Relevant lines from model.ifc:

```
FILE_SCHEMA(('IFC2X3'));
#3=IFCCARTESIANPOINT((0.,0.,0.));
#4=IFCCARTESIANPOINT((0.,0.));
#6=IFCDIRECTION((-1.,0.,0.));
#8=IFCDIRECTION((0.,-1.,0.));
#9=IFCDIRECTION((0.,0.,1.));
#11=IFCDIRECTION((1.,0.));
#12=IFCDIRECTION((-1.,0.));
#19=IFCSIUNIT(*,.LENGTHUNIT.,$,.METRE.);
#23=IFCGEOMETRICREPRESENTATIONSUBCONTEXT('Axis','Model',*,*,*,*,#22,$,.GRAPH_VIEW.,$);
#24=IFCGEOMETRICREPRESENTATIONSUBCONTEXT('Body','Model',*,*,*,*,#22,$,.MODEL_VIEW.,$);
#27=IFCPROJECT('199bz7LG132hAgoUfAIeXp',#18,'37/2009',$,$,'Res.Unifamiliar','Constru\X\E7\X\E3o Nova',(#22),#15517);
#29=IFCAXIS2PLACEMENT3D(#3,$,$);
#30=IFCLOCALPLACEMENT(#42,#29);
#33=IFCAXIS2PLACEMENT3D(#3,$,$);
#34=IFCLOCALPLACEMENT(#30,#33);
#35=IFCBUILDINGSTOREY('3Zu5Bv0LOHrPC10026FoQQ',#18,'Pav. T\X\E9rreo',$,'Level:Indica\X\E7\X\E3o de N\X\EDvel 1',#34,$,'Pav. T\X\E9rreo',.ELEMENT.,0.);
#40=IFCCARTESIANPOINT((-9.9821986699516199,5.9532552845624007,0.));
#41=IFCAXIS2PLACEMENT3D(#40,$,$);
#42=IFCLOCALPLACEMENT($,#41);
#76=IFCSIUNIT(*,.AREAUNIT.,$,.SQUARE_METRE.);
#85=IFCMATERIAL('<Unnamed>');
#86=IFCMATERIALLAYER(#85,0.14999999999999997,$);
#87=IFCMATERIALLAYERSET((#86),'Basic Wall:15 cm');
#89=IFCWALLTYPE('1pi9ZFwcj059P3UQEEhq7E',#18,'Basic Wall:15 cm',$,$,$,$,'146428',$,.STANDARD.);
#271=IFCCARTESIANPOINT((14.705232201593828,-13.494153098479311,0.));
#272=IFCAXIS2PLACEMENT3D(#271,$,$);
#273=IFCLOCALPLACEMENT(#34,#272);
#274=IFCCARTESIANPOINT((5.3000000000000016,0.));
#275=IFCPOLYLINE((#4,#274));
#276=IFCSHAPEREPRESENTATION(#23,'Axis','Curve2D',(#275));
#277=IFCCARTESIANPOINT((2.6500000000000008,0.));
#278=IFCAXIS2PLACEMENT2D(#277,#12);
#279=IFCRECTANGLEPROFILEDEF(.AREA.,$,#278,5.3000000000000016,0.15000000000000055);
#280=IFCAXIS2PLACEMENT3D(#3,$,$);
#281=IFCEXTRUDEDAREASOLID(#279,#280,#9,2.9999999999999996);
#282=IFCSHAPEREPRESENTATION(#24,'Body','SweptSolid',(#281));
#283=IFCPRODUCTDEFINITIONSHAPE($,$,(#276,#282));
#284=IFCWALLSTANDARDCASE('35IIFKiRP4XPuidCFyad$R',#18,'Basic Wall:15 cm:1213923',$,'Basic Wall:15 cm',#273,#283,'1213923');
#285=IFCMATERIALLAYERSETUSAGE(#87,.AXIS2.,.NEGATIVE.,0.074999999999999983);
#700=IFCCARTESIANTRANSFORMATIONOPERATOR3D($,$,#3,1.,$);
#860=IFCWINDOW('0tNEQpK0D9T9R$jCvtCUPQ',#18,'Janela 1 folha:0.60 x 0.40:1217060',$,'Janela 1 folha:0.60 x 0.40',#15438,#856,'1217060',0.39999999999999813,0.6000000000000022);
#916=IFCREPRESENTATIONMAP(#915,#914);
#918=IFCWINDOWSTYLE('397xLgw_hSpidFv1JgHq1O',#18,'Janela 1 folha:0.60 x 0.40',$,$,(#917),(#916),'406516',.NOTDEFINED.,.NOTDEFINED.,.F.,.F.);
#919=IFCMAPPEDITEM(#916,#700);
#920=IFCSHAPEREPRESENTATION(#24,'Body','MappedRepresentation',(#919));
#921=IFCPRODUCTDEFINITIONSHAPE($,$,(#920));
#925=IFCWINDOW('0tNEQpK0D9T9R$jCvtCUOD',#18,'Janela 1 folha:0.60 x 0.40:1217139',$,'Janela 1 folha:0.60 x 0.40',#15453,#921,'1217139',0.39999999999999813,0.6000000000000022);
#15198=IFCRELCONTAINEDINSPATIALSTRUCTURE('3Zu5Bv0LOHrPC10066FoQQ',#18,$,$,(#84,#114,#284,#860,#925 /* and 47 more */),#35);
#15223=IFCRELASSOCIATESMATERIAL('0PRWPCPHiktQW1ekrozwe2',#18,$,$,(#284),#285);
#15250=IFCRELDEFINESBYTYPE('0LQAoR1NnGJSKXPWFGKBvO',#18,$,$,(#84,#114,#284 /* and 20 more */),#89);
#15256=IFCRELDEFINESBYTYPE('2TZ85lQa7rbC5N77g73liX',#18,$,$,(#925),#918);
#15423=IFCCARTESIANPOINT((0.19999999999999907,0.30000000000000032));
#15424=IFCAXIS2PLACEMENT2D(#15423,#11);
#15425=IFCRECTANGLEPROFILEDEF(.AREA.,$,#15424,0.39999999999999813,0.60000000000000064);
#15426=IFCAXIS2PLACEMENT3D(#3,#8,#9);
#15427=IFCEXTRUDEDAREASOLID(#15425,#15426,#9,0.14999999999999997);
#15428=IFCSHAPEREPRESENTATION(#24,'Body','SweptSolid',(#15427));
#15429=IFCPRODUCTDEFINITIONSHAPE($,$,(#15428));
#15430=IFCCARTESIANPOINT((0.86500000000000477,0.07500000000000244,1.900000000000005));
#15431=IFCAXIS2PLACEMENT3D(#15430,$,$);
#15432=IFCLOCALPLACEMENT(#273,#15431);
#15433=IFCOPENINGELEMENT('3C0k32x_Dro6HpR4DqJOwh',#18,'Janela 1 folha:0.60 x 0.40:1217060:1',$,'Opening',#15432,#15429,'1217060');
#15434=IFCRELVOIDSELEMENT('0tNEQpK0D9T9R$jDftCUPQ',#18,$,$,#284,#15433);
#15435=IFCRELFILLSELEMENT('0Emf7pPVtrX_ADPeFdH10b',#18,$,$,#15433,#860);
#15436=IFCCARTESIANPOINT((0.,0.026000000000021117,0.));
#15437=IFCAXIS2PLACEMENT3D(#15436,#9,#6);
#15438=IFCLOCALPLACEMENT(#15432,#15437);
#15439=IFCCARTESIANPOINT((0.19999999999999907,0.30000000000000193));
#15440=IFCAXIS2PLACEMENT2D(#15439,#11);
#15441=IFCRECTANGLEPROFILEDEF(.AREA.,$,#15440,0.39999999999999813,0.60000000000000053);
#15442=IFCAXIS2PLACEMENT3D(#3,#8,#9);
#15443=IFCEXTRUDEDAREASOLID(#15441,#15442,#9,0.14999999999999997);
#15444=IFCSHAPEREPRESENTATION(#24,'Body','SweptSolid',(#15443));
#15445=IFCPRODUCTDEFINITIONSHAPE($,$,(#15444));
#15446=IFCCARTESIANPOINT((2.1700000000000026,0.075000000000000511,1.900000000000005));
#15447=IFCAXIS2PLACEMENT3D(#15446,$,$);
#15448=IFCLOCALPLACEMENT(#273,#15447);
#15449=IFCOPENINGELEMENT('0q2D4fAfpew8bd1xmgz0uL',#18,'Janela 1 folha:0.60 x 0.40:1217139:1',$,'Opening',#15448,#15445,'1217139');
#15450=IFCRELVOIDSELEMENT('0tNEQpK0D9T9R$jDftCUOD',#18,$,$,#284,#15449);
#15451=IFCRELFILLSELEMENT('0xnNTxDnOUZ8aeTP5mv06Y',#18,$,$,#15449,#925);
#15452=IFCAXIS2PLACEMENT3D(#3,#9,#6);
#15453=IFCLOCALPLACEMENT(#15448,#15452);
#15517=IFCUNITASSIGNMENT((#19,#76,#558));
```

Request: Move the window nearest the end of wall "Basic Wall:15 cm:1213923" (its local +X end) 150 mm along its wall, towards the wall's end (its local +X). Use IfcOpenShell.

```python
import ifcopenshell
import ifcopenshell.api.geometry
import ifcopenshell.util.placement
import ifcopenshell.util.unit

model = ifcopenshell.open("model.ifc")
unit_scale = ifcopenshell.util.unit.calculate_unit_scale(model)

window = model.by_guid("0tNEQpK0D9T9R$jCvtCUOD")
opening = window.FillsVoids[0].RelatingOpeningElement
wall = opening.VoidsElements[0].RelatingBuildingElement

wall_matrix = ifcopenshell.util.placement.get_local_placement(wall.ObjectPlacement)
shift = wall_matrix[:3, 0] * 0.15 / unit_scale
before = ifcopenshell.util.placement.get_local_placement(window.ObjectPlacement)[:3, 3].copy()

# The window is placed relative to its opening, so it follows when the opening moves.
matrix = ifcopenshell.util.placement.get_local_placement(opening.ObjectPlacement)
matrix[:3, 3] += shift
ifcopenshell.api.geometry.edit_object_placement(
    model, product=opening, matrix=matrix, is_si=False, should_transform_children=True
)

after = ifcopenshell.util.placement.get_local_placement(window.ObjectPlacement)[:3, 3]
print("window moved by", (after - before).round(3) + 0.0)

model.write("model_edited.ifc")
```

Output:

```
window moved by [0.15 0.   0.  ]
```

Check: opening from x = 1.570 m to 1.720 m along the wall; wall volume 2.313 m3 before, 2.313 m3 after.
